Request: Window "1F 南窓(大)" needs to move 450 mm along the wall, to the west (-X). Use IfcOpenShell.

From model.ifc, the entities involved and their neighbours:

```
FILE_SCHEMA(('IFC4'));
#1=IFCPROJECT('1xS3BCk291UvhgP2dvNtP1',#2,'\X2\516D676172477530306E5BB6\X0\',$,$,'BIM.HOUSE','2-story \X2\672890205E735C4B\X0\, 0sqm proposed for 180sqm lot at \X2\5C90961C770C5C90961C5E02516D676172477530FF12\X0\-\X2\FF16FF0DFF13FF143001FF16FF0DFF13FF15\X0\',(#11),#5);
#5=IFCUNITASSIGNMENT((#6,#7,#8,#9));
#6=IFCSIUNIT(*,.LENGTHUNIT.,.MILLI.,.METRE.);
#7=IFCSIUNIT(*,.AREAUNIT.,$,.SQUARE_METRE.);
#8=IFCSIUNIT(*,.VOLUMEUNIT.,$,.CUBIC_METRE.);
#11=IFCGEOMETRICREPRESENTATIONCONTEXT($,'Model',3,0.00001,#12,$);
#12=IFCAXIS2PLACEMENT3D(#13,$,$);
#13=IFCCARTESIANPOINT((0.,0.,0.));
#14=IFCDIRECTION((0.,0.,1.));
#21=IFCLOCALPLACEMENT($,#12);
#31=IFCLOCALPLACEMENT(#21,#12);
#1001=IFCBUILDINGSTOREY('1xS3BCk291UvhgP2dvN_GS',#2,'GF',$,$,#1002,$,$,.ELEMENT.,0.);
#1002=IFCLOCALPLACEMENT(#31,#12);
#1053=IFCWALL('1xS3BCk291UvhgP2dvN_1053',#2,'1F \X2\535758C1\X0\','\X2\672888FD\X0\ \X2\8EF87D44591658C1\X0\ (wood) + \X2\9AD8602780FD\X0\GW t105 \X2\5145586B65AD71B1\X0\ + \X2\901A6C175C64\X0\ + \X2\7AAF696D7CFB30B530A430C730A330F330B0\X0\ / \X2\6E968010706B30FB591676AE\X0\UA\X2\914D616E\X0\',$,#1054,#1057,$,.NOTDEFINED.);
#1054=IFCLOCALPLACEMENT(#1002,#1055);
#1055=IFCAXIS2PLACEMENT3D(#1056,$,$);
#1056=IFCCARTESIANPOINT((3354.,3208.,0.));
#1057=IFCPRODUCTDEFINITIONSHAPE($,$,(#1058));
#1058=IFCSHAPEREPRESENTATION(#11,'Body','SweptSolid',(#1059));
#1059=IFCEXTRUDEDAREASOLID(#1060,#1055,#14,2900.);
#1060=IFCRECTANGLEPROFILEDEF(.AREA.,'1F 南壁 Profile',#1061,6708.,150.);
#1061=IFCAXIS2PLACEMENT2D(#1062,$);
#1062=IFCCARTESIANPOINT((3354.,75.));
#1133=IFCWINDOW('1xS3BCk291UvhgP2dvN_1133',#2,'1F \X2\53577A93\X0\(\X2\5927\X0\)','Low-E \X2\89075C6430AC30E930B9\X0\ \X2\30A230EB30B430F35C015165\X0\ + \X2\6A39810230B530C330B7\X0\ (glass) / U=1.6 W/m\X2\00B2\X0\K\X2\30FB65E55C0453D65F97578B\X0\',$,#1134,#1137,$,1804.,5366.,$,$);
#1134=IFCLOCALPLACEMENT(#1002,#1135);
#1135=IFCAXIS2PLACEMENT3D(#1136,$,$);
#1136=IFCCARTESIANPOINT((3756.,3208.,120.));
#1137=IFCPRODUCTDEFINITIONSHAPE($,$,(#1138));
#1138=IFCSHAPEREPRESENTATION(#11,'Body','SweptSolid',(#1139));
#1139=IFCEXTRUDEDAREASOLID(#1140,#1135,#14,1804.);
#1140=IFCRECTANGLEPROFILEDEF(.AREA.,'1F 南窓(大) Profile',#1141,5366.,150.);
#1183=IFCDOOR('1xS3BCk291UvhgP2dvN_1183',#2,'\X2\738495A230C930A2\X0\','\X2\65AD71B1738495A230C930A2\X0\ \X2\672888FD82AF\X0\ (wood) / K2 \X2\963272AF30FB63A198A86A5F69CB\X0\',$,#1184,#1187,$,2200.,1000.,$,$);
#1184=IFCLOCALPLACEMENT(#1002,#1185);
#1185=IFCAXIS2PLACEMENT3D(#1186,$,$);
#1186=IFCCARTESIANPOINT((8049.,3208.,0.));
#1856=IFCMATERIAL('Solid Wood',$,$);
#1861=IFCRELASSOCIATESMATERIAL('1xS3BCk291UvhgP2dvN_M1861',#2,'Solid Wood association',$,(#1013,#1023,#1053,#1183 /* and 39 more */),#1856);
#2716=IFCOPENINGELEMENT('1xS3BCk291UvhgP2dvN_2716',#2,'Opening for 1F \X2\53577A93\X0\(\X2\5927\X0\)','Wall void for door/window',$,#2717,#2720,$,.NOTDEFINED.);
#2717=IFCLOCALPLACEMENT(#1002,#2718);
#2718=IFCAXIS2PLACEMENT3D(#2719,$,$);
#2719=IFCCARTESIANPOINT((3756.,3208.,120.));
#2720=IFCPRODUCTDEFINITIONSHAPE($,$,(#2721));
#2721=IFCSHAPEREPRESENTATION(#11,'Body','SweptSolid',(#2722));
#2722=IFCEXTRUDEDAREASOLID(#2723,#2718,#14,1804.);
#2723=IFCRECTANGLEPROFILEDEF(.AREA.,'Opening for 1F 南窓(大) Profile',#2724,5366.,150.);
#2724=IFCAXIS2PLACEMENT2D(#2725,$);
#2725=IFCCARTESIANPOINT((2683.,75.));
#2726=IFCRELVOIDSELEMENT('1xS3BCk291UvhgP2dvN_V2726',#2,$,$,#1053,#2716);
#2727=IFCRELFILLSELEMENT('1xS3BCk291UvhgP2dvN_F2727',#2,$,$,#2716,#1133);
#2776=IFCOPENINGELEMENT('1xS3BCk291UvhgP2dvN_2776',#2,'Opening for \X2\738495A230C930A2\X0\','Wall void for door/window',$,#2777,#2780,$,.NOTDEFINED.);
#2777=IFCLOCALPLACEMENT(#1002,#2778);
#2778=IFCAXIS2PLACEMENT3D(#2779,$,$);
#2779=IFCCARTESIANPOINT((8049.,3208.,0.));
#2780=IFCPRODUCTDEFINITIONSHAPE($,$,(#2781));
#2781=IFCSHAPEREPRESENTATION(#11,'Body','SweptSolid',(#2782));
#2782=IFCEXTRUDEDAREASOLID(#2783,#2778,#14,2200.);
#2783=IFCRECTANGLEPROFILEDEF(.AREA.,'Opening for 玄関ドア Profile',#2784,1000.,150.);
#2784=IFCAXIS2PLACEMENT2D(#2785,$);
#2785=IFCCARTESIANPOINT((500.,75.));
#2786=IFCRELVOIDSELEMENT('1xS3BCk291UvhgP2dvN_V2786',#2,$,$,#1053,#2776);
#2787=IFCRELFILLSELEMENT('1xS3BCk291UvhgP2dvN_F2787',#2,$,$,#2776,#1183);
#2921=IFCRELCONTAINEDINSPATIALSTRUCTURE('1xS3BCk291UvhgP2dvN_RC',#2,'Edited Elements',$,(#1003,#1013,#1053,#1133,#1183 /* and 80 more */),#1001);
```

```python
import ifcopenshell
import ifcopenshell.api.geometry
import ifcopenshell.util.placement
import ifcopenshell.util.unit

model = ifcopenshell.open("model.ifc")
unit_scale = ifcopenshell.util.unit.calculate_unit_scale(model)

window = model.by_id(1133)
opening = window.FillsVoids[0].RelatingOpeningElement
wall = opening.VoidsElements[0].RelatingBuildingElement

wall_matrix = ifcopenshell.util.placement.get_local_placement(wall.ObjectPlacement)
shift = wall_matrix[:3, 0] * -0.45 / unit_scale
before = ifcopenshell.util.placement.get_local_placement(window.ObjectPlacement)[:3, 3].copy()

# The window is not placed relative to its opening, so move both.
for product in (opening, window):
    matrix = ifcopenshell.util.placement.get_local_placement(product.ObjectPlacement)
    matrix[:3, 3] += shift
    ifcopenshell.api.geometry.edit_object_placement(model, product=product, matrix=matrix, is_si=False)

after = ifcopenshell.util.placement.get_local_placement(window.ObjectPlacement)[:3, 3]
print("window moved by", (after - before).round(3) + 0.0)

model.write("model_updated.ifc")
```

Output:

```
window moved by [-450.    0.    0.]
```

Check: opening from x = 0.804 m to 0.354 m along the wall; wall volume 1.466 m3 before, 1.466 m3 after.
